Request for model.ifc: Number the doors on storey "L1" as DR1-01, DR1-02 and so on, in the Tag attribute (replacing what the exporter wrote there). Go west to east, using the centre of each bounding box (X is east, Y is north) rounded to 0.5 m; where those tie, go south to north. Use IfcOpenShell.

First a look at what the model holds.

```python
import ifcopenshell
import ifcopenshell.util.element
import ifcopenshell.util.placement

model = ifcopenshell.open("model.ifc")
print(model.schema)
storey = next(s for s in model.by_type("IfcBuildingStorey") if s.Name == "L1")
doors = [e for e in ifcopenshell.util.element.get_decomposition(storey) if e.is_a("IfcDoor")]
for e in sorted(doors, key=lambda e: e.id()):
    origin = ifcopenshell.util.placement.get_local_placement(e.ObjectPlacement)[:3, 3]
    print(e.id(), e.Tag, e.Name, origin.round(2) + 0.0, sep=" | ")
```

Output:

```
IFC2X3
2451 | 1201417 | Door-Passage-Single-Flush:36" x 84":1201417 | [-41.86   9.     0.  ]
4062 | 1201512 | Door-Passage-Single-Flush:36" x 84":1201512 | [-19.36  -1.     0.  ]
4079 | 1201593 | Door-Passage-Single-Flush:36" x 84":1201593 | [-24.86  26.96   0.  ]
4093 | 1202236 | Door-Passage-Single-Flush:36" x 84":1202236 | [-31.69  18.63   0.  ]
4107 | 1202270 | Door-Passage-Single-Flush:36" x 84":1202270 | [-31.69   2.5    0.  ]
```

```python
import ifcopenshell
import ifcopenshell.geom
import ifcopenshell.util.element
import ifcopenshell.util.shape

model = ifcopenshell.open("model.ifc")
settings = ifcopenshell.geom.settings()
settings.set("use-world-coords", True)


def centre(element):
    shape = ifcopenshell.geom.create_shape(settings, element)
    return ifcopenshell.util.shape.get_bbox_centroid(shape.geometry)


storey = next(s for s in model.by_type("IfcBuildingStorey") if s.Name == "L1")
doors = [e for e in ifcopenshell.util.element.get_decomposition(storey) if e.is_a("IfcDoor")]

# Insertion points can sit at a corner or the storey origin, so sort by the geometry (in metres).
centres = {e: centre(e) for e in doors}
doors.sort(key=lambda e: (round(centres[e][0] / 0.5), centres[e][1]))

for i, e in enumerate(doors, start=1):
    number = f"DR1-{i:02d}"
    e.Tag = number
    print(e.id(), number)

model.write("model_v2.ifc")
```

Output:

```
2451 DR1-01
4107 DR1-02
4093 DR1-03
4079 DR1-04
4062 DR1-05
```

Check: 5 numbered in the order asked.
